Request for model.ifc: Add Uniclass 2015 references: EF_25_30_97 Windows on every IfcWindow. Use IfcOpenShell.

First a look at what the model holds.

```python
import ifcopenshell

model = ifcopenshell.open("model.ifc")
print(model.schema)
print("classifications:", [c.Name for c in model.by_type("IfcClassification")])
for ifc_class in ("IfcDoor", "IfcRoof", "IfcStair", "IfcWall", "IfcWindow"):
    print(ifc_class, len(model.by_type(ifc_class)))
```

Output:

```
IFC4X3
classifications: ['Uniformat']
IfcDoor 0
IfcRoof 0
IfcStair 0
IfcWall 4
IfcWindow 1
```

```python
import ifcopenshell
import ifcopenshell.api.classification

model = ifcopenshell.open("model.ifc")

system = ifcopenshell.api.classification.add_classification(model, classification="Uniclass 2015")

codes = {
    "IfcWindow": ("EF_25_30_97", "Windows"),
}
for ifc_class, (code, name) in codes.items():
    products = model.by_type(ifc_class)
    ifcopenshell.api.classification.add_reference(
        model, products=products, classification=system, identification=code, name=name
    )
    print(code, len(products))

model.write("model_rev.ifc")
```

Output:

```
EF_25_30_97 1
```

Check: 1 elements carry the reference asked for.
